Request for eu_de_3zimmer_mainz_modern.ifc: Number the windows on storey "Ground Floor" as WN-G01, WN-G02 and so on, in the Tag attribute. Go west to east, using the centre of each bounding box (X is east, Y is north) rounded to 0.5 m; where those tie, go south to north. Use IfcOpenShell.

First a look at what the model holds.

```python
import ifcopenshell
import ifcopenshell.util.element
import ifcopenshell.util.placement

model = ifcopenshell.open("eu_de_3zimmer_mainz_modern.ifc")
print(model.schema)
storey = next(s for s in model.by_type("IfcBuildingStorey") if s.Name == "Ground Floor")
windows = [e for e in ifcopenshell.util.element.get_decomposition(storey) if e.is_a("IfcWindow")]
for e in sorted(windows, key=lambda e: e.id()):
    origin = ifcopenshell.util.placement.get_local_placement(e.ObjectPlacement)[:3, 3]
    print(e.id(), e.Tag, e.Name, origin.round(2) + 0.0, sep=" | ")
```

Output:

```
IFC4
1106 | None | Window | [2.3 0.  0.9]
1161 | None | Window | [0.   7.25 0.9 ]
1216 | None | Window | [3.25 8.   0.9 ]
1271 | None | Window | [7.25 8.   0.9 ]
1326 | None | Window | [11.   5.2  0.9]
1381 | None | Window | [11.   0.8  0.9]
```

```python
import ifcopenshell
import ifcopenshell.geom
import ifcopenshell.util.element
import ifcopenshell.util.shape

model = ifcopenshell.open("eu_de_3zimmer_mainz_modern.ifc")
settings = ifcopenshell.geom.settings()
settings.set("use-world-coords", True)


def centre(element):
    shape = ifcopenshell.geom.create_shape(settings, element)
    return ifcopenshell.util.shape.get_bbox_centroid(shape.geometry)


storey = next(s for s in model.by_type("IfcBuildingStorey") if s.Name == "Ground Floor")
windows = [e for e in ifcopenshell.util.element.get_decomposition(storey) if e.is_a("IfcWindow")]

# Insertion points can sit at a corner or the storey origin, so sort by the geometry (in metres).
centres = {e: centre(e) for e in windows}
windows.sort(key=lambda e: (round(centres[e][0] / 0.5), centres[e][1]))

for i, e in enumerate(windows, start=1):
    number = f"WN-G{i:02d}"
    e.Tag = number
    print(e.id(), number)

model.write("eu_de_3zimmer_mainz_modern_edited.ifc")
```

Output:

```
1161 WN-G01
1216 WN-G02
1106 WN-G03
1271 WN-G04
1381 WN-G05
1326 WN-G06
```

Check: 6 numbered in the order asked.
